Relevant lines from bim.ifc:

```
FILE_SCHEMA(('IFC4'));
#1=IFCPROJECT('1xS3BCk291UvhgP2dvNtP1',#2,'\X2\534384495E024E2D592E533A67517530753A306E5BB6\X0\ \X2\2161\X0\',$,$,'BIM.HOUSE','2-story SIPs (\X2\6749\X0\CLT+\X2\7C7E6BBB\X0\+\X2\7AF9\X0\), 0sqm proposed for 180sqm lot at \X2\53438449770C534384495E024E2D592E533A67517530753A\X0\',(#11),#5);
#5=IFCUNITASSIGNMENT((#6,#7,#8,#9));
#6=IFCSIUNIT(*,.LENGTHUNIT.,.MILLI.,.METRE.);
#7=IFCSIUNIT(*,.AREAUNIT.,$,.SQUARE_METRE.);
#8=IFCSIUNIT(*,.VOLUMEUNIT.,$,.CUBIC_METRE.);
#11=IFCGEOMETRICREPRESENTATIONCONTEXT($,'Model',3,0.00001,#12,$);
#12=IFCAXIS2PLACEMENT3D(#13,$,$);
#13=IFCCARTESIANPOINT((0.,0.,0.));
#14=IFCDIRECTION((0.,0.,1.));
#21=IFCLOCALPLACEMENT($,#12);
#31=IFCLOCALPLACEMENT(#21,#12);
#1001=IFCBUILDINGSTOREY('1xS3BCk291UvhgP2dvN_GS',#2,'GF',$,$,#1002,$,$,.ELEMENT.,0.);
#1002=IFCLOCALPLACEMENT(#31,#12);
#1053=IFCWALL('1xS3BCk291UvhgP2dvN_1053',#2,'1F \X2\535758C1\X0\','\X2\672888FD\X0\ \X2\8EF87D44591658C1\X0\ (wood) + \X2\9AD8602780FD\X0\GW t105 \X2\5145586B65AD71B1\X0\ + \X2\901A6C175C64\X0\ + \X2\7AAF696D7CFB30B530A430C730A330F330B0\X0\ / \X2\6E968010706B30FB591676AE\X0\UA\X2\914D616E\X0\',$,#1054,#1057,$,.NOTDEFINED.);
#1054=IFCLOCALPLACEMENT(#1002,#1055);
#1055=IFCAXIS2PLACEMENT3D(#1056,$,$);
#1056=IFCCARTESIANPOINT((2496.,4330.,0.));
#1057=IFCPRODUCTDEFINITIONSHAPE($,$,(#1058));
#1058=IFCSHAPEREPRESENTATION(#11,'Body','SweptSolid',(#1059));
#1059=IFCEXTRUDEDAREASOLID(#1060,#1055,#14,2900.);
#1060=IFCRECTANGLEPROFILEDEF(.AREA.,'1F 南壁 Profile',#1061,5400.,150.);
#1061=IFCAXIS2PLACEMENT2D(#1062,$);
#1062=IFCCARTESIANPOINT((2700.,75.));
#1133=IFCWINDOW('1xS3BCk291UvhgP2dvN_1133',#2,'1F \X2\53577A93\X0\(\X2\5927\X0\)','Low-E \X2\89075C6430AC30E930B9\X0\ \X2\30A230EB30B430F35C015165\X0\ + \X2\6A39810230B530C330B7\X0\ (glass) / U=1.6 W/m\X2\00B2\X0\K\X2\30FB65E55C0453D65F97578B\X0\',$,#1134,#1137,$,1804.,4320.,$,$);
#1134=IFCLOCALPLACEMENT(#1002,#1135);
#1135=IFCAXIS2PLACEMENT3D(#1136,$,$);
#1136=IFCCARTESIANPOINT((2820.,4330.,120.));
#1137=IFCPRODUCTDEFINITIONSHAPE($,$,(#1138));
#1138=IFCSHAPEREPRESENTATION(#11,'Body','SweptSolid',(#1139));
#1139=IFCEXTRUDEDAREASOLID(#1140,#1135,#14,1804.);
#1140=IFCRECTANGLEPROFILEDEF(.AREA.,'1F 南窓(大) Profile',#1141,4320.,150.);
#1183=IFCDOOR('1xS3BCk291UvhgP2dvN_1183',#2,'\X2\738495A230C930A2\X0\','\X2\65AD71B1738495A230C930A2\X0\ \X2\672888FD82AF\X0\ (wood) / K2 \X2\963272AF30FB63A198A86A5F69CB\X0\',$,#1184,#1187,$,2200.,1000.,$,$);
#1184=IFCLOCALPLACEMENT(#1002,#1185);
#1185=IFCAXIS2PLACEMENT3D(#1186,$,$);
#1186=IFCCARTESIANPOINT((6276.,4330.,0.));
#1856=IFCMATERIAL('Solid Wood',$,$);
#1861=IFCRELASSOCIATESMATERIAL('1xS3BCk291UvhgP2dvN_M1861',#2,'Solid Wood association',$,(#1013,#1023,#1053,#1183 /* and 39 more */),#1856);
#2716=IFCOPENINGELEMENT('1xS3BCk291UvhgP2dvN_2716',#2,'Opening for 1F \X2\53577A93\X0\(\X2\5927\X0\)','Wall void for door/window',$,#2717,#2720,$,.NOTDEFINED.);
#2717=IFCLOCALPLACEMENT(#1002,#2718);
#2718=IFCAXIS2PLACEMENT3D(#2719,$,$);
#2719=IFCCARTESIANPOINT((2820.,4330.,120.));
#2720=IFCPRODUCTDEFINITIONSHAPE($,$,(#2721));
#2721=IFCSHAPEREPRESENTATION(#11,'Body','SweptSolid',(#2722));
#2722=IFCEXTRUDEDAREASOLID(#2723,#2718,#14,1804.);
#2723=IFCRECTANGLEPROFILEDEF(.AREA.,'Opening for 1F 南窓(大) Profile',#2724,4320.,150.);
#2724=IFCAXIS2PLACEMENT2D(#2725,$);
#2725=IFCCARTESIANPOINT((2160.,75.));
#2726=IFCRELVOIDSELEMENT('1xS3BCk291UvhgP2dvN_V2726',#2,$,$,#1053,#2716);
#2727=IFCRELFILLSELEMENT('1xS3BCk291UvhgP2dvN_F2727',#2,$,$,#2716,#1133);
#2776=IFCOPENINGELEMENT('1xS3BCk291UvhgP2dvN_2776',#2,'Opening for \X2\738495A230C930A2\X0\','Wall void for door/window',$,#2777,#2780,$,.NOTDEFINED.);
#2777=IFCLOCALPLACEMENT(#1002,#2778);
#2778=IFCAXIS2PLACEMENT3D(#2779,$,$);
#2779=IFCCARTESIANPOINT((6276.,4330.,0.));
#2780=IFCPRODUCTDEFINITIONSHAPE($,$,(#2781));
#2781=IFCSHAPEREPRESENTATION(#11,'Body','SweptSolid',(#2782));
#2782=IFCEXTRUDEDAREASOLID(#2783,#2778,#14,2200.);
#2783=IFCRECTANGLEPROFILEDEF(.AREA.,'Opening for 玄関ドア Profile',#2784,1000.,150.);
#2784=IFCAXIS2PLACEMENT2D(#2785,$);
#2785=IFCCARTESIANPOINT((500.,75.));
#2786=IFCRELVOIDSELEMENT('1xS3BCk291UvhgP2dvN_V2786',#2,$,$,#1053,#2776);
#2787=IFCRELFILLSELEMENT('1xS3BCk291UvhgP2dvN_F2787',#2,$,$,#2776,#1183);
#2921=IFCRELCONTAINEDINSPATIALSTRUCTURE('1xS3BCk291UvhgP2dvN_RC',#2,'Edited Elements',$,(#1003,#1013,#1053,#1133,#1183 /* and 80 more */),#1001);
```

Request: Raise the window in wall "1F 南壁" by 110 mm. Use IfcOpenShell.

```python
import numpy as np
import ifcopenshell
import ifcopenshell.api.geometry
import ifcopenshell.util.placement
import ifcopenshell.util.unit

model = ifcopenshell.open("bim.ifc")
unit_scale = ifcopenshell.util.unit.calculate_unit_scale(model)

window = model.by_id(1133)
opening = window.FillsVoids[0].RelatingOpeningElement
dz = 0.11 / unit_scale

shift = np.array([0.0, 0.0, dz])
# The window is not placed relative to its opening, so move both.
for product in (opening, window):
    matrix = ifcopenshell.util.placement.get_local_placement(product.ObjectPlacement)
    matrix[:3, 3] += shift
    ifcopenshell.api.geometry.edit_object_placement(model, product=product, matrix=matrix, is_si=False)

print(f"moved by {dz * unit_scale:+.3f} m")

model.write("bim_v2.ifc")
```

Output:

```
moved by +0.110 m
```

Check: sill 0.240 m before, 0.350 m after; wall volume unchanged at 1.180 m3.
